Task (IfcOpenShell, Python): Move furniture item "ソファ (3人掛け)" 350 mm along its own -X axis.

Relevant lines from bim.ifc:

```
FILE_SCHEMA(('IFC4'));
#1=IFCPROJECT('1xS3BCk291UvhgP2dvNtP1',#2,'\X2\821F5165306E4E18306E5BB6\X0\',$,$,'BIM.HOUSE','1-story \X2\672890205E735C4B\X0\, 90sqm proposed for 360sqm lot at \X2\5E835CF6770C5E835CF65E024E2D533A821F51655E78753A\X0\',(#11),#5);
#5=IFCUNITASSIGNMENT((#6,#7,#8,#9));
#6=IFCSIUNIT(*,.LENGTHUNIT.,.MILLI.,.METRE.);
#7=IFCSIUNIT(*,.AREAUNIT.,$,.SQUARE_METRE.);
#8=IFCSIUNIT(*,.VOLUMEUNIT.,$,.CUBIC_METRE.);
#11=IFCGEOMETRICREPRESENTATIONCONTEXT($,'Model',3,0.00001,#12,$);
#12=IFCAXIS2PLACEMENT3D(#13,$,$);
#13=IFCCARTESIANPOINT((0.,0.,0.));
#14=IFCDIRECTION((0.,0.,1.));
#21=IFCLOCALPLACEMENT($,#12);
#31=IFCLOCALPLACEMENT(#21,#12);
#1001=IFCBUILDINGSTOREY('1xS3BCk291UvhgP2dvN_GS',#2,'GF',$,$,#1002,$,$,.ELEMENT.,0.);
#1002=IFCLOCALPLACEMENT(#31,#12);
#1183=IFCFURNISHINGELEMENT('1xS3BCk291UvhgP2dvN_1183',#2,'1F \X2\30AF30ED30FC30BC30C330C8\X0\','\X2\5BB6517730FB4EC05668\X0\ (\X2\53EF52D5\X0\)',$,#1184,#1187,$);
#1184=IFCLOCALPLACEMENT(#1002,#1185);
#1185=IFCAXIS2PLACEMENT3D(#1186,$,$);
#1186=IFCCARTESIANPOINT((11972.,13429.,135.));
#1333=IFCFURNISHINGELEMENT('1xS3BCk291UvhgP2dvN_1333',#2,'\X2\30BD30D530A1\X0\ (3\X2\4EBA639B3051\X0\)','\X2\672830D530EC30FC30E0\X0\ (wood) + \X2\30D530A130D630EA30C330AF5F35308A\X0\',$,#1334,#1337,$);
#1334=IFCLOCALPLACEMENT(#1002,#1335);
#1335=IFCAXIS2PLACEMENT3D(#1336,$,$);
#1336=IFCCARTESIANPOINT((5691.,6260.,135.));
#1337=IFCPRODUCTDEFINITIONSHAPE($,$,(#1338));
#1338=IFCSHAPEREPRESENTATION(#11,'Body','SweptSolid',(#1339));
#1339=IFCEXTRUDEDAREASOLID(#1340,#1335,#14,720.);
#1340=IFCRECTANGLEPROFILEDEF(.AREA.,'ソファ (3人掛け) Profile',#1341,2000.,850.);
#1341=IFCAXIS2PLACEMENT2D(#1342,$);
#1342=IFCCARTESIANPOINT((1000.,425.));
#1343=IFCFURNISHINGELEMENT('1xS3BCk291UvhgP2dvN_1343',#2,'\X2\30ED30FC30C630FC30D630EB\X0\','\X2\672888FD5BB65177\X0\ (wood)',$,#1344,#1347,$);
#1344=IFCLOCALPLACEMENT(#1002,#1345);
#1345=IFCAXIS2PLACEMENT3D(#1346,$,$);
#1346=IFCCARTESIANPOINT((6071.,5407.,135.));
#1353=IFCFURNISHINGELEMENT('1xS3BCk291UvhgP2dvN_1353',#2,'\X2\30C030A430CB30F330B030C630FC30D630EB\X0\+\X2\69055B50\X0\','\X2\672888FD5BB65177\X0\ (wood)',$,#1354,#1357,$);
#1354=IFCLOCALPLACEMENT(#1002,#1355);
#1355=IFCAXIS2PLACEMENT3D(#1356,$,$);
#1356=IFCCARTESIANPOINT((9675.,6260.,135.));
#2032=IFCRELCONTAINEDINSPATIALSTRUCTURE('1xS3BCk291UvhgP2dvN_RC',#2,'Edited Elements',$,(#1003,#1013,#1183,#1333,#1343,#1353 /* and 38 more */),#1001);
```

```python
import ifcopenshell
import ifcopenshell.api.geometry
import ifcopenshell.util.placement
import ifcopenshell.util.unit

model = ifcopenshell.open("bim.ifc")
unit_scale = ifcopenshell.util.unit.calculate_unit_scale(model)

item = model.by_guid("1xS3BCk291UvhgP2dvN_1333")
matrix = ifcopenshell.util.placement.get_local_placement(item.ObjectPlacement)
matrix[:3, 3] -= matrix[:3, 0] * 0.35 / unit_scale
ifcopenshell.api.geometry.edit_object_placement(model, product=item, matrix=matrix, is_si=False)

print(ifcopenshell.util.placement.get_local_placement(item.ObjectPlacement).round(3) + 0.0)

model.write("bim_v2.ifc")
```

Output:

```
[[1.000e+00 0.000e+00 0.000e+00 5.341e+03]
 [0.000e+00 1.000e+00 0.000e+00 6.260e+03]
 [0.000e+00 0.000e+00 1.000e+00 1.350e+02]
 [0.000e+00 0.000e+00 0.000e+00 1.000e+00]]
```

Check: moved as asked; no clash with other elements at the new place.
